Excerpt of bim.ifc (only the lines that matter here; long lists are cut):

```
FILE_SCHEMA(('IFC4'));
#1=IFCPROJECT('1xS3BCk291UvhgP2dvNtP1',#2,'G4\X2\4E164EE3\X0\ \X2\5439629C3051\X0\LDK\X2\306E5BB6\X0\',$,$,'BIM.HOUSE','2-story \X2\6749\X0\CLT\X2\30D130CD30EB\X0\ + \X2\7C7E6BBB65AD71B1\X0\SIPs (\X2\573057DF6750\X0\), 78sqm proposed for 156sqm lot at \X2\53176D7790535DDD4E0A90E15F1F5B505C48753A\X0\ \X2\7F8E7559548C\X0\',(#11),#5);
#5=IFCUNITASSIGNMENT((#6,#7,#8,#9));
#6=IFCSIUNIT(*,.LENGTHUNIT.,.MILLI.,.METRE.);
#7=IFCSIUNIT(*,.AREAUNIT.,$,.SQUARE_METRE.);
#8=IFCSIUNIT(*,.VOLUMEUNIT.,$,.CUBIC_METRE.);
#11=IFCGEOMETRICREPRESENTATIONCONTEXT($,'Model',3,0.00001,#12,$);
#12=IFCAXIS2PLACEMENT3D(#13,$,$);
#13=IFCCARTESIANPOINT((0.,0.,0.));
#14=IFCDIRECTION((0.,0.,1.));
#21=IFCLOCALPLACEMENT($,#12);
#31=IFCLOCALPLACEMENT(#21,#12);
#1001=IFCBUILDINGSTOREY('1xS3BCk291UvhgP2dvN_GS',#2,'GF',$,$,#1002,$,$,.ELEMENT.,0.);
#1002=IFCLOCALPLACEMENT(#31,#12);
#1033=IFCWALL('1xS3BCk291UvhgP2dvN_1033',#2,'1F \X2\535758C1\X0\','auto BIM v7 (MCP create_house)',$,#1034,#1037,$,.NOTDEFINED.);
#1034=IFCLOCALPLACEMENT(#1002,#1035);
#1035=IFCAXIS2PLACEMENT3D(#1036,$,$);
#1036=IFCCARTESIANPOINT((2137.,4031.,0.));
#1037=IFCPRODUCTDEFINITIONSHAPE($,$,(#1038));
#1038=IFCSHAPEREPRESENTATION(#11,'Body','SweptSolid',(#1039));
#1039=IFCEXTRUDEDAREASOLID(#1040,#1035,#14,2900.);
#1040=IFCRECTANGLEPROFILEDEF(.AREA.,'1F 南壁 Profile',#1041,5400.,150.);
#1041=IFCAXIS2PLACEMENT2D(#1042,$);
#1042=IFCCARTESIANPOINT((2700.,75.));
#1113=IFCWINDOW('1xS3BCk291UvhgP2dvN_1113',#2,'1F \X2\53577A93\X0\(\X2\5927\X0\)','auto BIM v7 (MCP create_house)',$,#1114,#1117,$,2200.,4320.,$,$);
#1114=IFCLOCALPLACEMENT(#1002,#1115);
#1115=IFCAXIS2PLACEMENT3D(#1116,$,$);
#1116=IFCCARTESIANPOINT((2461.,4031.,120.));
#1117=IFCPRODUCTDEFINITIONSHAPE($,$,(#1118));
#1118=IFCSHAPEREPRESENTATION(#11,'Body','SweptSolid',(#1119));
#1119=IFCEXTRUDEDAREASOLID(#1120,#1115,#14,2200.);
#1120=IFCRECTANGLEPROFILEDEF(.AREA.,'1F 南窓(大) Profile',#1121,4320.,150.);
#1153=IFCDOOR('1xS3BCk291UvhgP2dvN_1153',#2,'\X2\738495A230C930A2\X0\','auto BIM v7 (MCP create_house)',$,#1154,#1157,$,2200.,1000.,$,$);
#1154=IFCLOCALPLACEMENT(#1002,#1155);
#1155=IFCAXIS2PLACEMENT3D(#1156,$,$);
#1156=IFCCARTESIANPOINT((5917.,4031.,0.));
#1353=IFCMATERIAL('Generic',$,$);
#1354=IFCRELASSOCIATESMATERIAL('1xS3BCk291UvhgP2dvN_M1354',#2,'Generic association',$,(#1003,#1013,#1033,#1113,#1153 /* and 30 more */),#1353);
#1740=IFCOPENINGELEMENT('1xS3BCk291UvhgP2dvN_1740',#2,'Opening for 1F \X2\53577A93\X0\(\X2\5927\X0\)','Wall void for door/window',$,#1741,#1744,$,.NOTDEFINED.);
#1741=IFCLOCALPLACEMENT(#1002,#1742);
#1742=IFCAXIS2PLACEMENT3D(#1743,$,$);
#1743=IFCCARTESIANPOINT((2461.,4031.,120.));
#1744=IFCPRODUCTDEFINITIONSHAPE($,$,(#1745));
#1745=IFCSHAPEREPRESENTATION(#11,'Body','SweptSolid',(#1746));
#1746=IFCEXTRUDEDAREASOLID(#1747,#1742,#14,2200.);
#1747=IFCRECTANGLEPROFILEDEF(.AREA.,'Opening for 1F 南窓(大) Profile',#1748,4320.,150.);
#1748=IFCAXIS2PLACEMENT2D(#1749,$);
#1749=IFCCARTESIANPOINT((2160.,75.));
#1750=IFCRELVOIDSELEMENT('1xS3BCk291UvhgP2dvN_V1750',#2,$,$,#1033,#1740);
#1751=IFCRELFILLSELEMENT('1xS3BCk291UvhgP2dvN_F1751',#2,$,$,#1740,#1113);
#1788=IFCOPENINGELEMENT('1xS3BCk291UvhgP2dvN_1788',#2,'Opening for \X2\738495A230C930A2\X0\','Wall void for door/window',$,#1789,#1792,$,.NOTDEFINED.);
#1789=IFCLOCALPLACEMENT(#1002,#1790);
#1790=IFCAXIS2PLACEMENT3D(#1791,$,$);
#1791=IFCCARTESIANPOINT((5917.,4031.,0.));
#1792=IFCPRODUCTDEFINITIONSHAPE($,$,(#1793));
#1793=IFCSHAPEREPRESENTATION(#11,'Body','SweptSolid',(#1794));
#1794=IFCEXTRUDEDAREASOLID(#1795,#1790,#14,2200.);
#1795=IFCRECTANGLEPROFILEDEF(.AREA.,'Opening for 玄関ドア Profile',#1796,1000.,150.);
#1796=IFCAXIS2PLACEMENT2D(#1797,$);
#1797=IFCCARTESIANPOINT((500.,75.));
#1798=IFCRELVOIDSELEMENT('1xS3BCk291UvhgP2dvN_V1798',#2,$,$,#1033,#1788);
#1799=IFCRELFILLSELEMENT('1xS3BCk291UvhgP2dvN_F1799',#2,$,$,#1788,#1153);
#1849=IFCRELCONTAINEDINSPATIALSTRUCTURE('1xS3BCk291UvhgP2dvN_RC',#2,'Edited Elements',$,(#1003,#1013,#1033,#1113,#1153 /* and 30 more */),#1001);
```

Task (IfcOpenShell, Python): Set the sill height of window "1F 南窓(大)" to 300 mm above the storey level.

```python
import numpy as np
import ifcopenshell
import ifcopenshell.api.geometry
import ifcopenshell.geom
import ifcopenshell.util.element
import ifcopenshell.util.placement
import ifcopenshell.util.shape
import ifcopenshell.util.unit

model = ifcopenshell.open("bim.ifc")
unit_scale = ifcopenshell.util.unit.calculate_unit_scale(model)

window = model.by_guid("1xS3BCk291UvhgP2dvN_1113")
opening = window.FillsVoids[0].RelatingOpeningElement
storey = ifcopenshell.util.element.get_container(window, ifc_class="IfcBuildingStorey")
level = ifcopenshell.util.placement.get_local_placement(storey.ObjectPlacement)[2, 3]

# The opening's origin need not be at the sill, so measure its lowest point.
shape = ifcopenshell.geom.create_shape(ifcopenshell.geom.settings(), opening)
bottom = ifcopenshell.util.shape.get_shape_bottom_elevation(shape, shape.geometry) / unit_scale
dz = level + 300.0 - bottom

shift = np.array([0.0, 0.0, dz])
# The window is not placed relative to its opening, so move both.
for product in (opening, window):
    matrix = ifcopenshell.util.placement.get_local_placement(product.ObjectPlacement)
    matrix[:3, 3] += shift
    ifcopenshell.api.geometry.edit_object_placement(model, product=product, matrix=matrix, is_si=False)

print(f"moved by {dz * unit_scale:+.3f} m")

model.write("bim_updated.ifc")
```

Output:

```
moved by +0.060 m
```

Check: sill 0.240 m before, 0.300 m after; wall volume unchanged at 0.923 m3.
